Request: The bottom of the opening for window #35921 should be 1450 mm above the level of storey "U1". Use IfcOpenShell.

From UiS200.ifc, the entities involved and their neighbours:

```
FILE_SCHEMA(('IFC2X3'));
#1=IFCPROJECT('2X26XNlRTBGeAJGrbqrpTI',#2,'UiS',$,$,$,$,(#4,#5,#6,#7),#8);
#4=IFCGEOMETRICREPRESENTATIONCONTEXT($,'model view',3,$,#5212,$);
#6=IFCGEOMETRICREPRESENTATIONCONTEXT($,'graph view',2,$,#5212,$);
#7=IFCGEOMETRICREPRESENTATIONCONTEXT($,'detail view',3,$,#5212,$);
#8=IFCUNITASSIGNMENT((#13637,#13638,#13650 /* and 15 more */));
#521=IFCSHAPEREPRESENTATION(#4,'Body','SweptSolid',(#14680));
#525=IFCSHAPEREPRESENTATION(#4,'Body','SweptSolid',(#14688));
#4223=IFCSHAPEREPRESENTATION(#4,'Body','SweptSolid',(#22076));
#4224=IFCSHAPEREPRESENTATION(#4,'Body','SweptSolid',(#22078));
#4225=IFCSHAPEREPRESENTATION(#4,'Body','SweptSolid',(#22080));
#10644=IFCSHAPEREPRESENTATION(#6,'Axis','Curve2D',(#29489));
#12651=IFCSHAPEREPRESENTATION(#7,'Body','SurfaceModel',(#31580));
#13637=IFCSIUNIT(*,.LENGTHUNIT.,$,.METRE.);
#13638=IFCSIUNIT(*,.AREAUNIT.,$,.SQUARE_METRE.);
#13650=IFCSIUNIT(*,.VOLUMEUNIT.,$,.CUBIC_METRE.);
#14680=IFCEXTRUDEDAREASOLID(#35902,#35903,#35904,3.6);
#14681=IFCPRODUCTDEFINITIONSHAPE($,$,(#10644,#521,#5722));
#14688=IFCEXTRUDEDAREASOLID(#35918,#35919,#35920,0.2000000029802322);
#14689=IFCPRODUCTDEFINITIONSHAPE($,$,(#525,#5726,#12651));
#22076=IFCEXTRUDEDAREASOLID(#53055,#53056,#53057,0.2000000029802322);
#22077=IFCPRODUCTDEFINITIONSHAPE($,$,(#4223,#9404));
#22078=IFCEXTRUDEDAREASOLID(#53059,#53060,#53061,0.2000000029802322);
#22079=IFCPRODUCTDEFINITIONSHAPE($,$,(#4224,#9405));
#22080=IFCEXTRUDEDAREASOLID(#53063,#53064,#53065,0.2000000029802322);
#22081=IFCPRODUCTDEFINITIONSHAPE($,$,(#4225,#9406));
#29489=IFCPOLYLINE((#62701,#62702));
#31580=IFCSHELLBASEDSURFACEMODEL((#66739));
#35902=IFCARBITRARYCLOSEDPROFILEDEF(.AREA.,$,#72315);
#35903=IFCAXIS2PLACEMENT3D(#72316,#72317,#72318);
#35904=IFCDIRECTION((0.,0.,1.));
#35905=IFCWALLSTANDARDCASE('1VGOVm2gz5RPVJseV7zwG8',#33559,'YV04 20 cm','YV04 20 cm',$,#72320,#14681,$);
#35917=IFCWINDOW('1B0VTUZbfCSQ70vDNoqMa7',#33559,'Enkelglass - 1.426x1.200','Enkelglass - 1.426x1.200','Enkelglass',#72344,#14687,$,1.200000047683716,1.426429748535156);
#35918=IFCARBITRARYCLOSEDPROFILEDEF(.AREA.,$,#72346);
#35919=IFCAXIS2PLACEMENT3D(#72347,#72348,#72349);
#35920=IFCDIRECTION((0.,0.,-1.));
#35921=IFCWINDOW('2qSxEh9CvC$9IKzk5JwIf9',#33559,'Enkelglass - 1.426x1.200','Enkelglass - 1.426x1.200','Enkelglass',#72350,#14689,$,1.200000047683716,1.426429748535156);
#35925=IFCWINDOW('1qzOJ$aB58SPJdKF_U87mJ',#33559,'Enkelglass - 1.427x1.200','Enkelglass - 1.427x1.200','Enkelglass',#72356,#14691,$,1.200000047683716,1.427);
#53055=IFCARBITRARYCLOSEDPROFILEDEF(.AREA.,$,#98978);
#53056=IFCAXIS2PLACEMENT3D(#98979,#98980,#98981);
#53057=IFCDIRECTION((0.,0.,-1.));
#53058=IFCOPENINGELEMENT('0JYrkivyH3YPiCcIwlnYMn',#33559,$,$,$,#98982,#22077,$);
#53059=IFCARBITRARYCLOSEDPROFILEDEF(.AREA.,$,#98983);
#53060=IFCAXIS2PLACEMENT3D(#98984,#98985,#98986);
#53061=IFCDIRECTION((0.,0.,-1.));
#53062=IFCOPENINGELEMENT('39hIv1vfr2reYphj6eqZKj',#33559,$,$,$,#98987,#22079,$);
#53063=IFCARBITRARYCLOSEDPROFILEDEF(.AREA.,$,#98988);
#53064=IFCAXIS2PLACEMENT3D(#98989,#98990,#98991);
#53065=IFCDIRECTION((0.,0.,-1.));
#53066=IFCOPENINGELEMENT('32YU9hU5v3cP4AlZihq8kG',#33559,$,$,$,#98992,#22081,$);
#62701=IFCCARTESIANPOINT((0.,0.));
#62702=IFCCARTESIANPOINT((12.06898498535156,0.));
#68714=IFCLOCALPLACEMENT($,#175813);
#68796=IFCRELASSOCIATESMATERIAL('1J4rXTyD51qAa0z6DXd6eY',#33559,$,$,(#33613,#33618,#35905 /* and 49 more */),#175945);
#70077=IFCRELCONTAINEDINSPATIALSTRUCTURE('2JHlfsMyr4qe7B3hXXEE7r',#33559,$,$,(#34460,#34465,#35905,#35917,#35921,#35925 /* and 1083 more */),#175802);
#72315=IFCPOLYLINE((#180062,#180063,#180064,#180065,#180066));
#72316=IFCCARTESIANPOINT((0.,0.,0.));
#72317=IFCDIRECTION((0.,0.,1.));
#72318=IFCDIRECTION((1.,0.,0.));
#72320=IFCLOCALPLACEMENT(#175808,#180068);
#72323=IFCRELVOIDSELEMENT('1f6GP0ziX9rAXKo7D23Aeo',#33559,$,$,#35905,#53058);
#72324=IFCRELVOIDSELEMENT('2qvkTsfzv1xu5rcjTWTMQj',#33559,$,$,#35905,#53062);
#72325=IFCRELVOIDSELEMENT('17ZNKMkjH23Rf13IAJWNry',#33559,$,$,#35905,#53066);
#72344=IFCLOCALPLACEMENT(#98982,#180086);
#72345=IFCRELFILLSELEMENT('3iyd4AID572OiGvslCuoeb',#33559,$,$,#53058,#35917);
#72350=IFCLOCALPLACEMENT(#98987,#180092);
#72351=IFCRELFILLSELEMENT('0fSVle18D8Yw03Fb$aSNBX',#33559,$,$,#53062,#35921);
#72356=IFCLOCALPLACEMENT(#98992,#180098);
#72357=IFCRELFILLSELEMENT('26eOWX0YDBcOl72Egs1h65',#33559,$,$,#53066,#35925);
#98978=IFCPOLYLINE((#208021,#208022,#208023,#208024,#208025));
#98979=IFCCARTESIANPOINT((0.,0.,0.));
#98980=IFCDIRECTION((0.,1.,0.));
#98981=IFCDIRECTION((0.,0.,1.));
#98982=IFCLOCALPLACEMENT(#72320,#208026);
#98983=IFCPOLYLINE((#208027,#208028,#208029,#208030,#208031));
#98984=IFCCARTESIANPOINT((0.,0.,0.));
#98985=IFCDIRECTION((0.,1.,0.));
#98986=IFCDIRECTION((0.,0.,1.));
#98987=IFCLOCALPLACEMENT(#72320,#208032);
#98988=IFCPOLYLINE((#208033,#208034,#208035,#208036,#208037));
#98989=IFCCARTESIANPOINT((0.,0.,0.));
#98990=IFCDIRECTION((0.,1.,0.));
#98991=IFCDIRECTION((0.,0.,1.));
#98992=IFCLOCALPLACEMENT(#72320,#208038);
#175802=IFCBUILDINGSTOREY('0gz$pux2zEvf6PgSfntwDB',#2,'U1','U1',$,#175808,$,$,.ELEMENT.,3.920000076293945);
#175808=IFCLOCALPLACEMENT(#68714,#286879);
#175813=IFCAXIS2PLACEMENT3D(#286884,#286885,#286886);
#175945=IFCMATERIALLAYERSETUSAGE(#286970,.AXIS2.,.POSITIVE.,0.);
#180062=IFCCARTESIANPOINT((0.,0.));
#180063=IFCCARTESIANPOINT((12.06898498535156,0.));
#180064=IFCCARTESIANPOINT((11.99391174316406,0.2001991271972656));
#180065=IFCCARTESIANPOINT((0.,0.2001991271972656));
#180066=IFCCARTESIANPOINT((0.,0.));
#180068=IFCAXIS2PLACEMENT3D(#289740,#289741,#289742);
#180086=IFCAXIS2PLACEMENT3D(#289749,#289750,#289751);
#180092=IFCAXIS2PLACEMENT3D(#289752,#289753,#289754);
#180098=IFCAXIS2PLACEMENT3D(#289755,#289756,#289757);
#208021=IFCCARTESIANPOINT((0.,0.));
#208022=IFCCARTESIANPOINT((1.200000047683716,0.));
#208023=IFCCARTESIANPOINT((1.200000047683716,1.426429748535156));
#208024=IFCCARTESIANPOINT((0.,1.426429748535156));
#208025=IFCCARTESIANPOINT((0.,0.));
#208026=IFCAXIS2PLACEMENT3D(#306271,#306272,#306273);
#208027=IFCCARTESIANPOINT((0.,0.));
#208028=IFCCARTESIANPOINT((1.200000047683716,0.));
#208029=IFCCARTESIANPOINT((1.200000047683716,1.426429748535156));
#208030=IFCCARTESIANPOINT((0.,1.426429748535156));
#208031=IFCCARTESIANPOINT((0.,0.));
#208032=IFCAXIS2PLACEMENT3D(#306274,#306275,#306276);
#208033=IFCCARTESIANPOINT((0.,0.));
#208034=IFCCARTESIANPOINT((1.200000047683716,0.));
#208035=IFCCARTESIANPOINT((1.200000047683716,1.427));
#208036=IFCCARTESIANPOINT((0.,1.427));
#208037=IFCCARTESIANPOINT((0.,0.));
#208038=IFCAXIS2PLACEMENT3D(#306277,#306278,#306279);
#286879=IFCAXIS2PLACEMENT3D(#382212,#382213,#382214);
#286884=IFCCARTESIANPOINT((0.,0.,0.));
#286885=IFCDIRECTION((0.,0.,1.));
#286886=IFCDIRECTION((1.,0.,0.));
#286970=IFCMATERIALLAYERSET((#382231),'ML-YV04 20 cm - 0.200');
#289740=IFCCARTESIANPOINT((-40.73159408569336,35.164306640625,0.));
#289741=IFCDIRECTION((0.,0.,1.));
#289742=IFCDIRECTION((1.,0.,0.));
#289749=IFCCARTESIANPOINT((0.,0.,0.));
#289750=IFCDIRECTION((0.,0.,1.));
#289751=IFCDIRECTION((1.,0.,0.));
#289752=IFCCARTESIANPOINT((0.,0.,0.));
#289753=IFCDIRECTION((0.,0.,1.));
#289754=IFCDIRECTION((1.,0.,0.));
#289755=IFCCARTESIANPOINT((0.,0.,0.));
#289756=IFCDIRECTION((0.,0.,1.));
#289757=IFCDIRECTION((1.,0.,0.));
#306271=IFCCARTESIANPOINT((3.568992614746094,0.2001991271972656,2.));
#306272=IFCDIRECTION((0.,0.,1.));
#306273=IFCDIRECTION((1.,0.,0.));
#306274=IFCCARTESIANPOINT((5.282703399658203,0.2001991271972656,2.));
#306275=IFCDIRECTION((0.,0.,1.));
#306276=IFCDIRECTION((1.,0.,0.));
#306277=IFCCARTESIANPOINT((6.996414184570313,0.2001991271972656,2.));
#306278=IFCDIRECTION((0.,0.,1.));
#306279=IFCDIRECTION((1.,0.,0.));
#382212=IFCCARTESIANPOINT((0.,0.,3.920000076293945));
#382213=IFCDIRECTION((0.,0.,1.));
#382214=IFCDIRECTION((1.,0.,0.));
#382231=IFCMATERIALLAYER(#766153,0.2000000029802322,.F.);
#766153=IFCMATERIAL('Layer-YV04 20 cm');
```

```python
import numpy as np
import ifcopenshell
import ifcopenshell.api.geometry
import ifcopenshell.geom
import ifcopenshell.util.element
import ifcopenshell.util.placement
import ifcopenshell.util.shape
import ifcopenshell.util.unit

model = ifcopenshell.open("UiS200.ifc")
unit_scale = ifcopenshell.util.unit.calculate_unit_scale(model)

window = model.by_guid("2qSxEh9CvC$9IKzk5JwIf9")
opening = window.FillsVoids[0].RelatingOpeningElement
storey = ifcopenshell.util.element.get_container(window, ifc_class="IfcBuildingStorey")
level = ifcopenshell.util.placement.get_local_placement(storey.ObjectPlacement)[2, 3]

# The opening's origin need not be at the sill, so measure its lowest point.
shape = ifcopenshell.geom.create_shape(ifcopenshell.geom.settings(), opening)
bottom = ifcopenshell.util.shape.get_shape_bottom_elevation(shape, shape.geometry) / unit_scale
dz = level + 1.45 - bottom

shift = np.array([0.0, 0.0, dz])
# The window is placed relative to its opening, so it follows when the opening moves.
matrix = ifcopenshell.util.placement.get_local_placement(opening.ObjectPlacement)
matrix[:3, 3] += shift
ifcopenshell.api.geometry.edit_object_placement(
    model, product=opening, matrix=matrix, is_si=False, should_transform_children=True
)

print(f"moved by {dz * unit_scale:+.3f} m")

model.write("UiS200_updated.ifc")
```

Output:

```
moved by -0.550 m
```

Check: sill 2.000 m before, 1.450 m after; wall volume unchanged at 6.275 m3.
